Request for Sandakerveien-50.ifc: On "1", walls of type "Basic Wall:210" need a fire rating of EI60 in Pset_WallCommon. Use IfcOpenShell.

First a look at what the model holds.

```python
import ifcopenshell
import ifcopenshell.util.element

model = ifcopenshell.open("Sandakerveien-50.ifc")
print(model.schema)
storey = next(s for s in model.by_type("IfcBuildingStorey") if s.Name == "1")
walls = [e for e in ifcopenshell.util.element.get_decomposition(storey) if e.is_a("IfcWall")]
seen = {}
for e in walls:
    element_type = ifcopenshell.util.element.get_type(e)
    key = (element_type.Name if element_type != e and element_type else None, ifcopenshell.util.element.get_pset(e, "Pset_WallCommon", "FireRating"))
    seen[key] = seen.get(key, 0) + 1
for (name, value), count in sorted(seen.items(), key=str):
    print(count, "x", name, "|", value)
```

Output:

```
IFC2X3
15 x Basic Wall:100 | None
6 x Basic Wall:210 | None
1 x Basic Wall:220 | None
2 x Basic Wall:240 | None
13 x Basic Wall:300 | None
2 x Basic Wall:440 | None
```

```python
import ifcopenshell
import ifcopenshell.api.pset
import ifcopenshell.util.element

model = ifcopenshell.open("Sandakerveien-50.ifc")

storey = next(s for s in model.by_type("IfcBuildingStorey") if s.Name == "1")
walls = [e for e in ifcopenshell.util.element.get_decomposition(storey) if e.is_a("IfcWall")]

count = 0
for e in walls:
    element_type = ifcopenshell.util.element.get_type(e)
    if element_type in (None, e) or element_type.Name != "Basic Wall:210":
        continue
    # add_pset returns the element's existing set when there is one.
    pset = ifcopenshell.api.pset.add_pset(model, product=e, name="Pset_WallCommon")
    ifcopenshell.api.pset.edit_pset(model, pset=pset, properties={"FireRating": "EI60"})
    count += 1

print(count, "walls updated")

model.write("Sandakerveien-50-out.ifc")
```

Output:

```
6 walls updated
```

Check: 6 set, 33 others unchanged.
